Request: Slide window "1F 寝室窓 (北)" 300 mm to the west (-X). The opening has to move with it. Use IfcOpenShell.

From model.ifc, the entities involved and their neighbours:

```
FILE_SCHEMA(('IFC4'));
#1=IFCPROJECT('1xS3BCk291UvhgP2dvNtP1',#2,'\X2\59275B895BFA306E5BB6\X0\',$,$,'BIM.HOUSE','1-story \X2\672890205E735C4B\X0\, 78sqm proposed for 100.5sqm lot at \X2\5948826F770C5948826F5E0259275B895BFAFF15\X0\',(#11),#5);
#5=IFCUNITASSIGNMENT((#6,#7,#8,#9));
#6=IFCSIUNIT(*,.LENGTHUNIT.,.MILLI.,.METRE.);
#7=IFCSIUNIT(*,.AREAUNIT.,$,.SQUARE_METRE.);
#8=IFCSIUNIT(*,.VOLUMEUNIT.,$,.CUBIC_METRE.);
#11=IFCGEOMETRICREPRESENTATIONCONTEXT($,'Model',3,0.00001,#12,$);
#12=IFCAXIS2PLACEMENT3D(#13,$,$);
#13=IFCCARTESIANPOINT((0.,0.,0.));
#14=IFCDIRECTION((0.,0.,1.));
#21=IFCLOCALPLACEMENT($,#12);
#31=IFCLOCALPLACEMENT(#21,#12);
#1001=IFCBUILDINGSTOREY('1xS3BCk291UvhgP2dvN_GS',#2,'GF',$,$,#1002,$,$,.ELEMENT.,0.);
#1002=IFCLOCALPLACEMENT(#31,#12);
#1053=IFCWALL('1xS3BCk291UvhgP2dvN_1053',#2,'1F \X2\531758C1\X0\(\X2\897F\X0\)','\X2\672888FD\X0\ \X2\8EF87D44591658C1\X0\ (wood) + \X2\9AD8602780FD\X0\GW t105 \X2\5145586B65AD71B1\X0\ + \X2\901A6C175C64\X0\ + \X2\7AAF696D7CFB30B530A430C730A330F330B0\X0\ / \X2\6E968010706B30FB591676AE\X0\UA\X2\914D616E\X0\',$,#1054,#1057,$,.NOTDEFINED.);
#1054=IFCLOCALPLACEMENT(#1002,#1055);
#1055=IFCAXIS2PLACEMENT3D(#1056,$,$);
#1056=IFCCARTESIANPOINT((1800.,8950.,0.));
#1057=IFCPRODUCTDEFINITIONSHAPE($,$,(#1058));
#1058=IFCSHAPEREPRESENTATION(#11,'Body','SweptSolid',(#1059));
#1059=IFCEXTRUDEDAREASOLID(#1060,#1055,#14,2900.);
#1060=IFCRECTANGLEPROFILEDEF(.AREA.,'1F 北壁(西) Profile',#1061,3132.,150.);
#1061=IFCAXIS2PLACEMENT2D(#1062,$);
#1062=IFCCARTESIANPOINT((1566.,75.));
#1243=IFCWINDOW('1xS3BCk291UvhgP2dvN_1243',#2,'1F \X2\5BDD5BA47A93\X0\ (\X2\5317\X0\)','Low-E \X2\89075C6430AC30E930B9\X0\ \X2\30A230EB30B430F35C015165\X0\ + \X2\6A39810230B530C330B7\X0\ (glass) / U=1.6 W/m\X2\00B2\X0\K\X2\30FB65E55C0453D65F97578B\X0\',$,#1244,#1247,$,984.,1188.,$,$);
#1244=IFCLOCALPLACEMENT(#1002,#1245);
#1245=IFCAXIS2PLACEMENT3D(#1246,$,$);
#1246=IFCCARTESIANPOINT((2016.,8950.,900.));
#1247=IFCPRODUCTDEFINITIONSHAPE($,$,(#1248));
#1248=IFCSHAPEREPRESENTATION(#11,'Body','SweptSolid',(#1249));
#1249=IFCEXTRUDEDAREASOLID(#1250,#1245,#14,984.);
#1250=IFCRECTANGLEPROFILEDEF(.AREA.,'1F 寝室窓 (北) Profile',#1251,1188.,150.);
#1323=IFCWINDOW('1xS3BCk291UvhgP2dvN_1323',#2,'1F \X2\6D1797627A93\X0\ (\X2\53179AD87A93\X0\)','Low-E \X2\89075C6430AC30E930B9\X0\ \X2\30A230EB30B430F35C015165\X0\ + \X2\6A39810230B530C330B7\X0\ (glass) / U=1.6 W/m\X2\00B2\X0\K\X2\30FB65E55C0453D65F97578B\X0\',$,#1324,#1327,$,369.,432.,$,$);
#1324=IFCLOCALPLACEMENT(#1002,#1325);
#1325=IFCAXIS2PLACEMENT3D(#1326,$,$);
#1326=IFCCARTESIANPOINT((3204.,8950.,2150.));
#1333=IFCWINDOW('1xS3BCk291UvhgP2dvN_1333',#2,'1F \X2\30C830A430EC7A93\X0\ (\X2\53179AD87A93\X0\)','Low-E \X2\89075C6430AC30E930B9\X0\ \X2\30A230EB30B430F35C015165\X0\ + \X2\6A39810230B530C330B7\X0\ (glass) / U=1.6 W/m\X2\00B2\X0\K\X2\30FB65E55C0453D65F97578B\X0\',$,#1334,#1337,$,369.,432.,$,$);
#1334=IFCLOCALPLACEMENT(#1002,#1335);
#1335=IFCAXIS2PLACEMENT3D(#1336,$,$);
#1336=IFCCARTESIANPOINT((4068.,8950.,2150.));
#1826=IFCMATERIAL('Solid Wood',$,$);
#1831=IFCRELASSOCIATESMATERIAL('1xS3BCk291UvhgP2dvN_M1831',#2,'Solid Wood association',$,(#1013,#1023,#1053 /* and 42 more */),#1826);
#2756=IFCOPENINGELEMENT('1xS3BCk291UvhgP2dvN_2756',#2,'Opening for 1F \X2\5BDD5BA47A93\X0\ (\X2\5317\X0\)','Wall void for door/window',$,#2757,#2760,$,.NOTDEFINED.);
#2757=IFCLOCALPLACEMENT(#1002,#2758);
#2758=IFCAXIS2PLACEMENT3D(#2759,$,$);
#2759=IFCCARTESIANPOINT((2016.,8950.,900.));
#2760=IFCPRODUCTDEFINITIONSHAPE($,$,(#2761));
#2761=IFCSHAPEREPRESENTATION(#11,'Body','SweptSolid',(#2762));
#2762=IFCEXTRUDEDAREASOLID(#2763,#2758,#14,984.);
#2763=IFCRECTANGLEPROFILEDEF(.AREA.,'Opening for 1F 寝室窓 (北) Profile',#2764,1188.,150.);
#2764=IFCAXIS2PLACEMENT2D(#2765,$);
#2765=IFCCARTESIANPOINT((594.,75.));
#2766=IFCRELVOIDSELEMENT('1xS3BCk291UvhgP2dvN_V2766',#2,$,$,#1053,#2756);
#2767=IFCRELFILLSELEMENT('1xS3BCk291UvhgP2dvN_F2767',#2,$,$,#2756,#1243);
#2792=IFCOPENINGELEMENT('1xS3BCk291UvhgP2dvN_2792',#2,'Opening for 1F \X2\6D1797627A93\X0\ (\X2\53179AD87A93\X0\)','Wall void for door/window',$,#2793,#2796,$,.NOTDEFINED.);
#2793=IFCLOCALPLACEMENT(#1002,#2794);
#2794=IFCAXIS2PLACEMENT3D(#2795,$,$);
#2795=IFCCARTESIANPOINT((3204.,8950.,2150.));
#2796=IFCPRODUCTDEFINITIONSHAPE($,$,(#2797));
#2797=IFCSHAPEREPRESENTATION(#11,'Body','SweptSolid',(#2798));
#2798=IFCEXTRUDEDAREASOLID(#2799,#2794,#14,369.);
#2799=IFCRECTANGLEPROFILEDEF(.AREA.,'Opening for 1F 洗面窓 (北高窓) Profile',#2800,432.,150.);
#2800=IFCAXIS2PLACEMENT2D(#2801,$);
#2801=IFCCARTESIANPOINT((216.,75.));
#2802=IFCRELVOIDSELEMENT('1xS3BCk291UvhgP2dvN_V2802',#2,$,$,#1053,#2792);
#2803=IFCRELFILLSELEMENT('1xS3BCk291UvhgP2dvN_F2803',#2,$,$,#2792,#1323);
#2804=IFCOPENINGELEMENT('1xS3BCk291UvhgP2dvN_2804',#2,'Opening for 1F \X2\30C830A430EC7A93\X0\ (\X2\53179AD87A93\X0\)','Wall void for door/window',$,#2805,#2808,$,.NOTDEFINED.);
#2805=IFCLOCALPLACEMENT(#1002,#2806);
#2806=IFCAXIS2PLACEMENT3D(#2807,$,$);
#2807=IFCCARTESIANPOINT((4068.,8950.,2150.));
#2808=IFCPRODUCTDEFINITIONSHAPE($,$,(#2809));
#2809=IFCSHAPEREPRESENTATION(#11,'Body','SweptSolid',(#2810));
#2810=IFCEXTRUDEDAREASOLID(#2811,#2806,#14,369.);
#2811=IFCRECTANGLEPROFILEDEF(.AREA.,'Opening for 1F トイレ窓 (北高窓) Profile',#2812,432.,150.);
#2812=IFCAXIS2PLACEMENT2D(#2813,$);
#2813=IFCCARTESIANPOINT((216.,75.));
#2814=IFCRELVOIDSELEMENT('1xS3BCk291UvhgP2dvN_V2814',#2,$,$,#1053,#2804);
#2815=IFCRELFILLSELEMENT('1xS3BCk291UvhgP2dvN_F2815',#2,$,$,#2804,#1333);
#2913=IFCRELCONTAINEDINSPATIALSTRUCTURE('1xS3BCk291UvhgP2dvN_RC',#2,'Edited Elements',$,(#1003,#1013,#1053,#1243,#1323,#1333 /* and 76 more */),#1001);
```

```python
import ifcopenshell
import ifcopenshell.api.geometry
import ifcopenshell.util.placement
import ifcopenshell.util.unit

model = ifcopenshell.open("model.ifc")
unit_scale = ifcopenshell.util.unit.calculate_unit_scale(model)

window = model.by_guid("1xS3BCk291UvhgP2dvN_1243")
opening = window.FillsVoids[0].RelatingOpeningElement
wall = opening.VoidsElements[0].RelatingBuildingElement

wall_matrix = ifcopenshell.util.placement.get_local_placement(wall.ObjectPlacement)
shift = wall_matrix[:3, 0] * -0.3 / unit_scale
before = ifcopenshell.util.placement.get_local_placement(window.ObjectPlacement)[:3, 3].copy()

# The window is not placed relative to its opening, so move both.
for product in (opening, window):
    matrix = ifcopenshell.util.placement.get_local_placement(product.ObjectPlacement)
    matrix[:3, 3] += shift
    ifcopenshell.api.geometry.edit_object_placement(model, product=product, matrix=matrix, is_si=False)

after = ifcopenshell.util.placement.get_local_placement(window.ObjectPlacement)[:3, 3]
print("window moved by", (after - before).round(3) + 0.0)

model.write("model-out.ifc")
```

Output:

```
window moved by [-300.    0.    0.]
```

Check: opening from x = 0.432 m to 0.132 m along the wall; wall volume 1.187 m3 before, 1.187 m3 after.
